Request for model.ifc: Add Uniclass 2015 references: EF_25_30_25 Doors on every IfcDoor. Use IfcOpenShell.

First a look at what the model holds.

```python
import ifcopenshell

model = ifcopenshell.open("model.ifc")
print(model.schema)
print("classifications:", [c.Name for c in model.by_type("IfcClassification")])
for ifc_class in ("IfcDoor", "IfcRoof", "IfcStair", "IfcWall", "IfcWindow"):
    print(ifc_class, len(model.by_type(ifc_class)))
```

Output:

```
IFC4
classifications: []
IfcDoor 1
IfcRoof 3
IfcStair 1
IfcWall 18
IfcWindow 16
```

```python
import ifcopenshell
import ifcopenshell.api.classification

model = ifcopenshell.open("model.ifc")

system = ifcopenshell.api.classification.add_classification(model, classification="Uniclass 2015")

codes = {
    "IfcDoor": ("EF_25_30_25", "Doors"),
}
for ifc_class, (code, name) in codes.items():
    products = model.by_type(ifc_class)
    ifcopenshell.api.classification.add_reference(
        model, products=products, classification=system, identification=code, name=name
    )
    print(code, len(products))

model.write("model_edited.ifc")
```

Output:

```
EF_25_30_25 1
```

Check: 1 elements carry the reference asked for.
